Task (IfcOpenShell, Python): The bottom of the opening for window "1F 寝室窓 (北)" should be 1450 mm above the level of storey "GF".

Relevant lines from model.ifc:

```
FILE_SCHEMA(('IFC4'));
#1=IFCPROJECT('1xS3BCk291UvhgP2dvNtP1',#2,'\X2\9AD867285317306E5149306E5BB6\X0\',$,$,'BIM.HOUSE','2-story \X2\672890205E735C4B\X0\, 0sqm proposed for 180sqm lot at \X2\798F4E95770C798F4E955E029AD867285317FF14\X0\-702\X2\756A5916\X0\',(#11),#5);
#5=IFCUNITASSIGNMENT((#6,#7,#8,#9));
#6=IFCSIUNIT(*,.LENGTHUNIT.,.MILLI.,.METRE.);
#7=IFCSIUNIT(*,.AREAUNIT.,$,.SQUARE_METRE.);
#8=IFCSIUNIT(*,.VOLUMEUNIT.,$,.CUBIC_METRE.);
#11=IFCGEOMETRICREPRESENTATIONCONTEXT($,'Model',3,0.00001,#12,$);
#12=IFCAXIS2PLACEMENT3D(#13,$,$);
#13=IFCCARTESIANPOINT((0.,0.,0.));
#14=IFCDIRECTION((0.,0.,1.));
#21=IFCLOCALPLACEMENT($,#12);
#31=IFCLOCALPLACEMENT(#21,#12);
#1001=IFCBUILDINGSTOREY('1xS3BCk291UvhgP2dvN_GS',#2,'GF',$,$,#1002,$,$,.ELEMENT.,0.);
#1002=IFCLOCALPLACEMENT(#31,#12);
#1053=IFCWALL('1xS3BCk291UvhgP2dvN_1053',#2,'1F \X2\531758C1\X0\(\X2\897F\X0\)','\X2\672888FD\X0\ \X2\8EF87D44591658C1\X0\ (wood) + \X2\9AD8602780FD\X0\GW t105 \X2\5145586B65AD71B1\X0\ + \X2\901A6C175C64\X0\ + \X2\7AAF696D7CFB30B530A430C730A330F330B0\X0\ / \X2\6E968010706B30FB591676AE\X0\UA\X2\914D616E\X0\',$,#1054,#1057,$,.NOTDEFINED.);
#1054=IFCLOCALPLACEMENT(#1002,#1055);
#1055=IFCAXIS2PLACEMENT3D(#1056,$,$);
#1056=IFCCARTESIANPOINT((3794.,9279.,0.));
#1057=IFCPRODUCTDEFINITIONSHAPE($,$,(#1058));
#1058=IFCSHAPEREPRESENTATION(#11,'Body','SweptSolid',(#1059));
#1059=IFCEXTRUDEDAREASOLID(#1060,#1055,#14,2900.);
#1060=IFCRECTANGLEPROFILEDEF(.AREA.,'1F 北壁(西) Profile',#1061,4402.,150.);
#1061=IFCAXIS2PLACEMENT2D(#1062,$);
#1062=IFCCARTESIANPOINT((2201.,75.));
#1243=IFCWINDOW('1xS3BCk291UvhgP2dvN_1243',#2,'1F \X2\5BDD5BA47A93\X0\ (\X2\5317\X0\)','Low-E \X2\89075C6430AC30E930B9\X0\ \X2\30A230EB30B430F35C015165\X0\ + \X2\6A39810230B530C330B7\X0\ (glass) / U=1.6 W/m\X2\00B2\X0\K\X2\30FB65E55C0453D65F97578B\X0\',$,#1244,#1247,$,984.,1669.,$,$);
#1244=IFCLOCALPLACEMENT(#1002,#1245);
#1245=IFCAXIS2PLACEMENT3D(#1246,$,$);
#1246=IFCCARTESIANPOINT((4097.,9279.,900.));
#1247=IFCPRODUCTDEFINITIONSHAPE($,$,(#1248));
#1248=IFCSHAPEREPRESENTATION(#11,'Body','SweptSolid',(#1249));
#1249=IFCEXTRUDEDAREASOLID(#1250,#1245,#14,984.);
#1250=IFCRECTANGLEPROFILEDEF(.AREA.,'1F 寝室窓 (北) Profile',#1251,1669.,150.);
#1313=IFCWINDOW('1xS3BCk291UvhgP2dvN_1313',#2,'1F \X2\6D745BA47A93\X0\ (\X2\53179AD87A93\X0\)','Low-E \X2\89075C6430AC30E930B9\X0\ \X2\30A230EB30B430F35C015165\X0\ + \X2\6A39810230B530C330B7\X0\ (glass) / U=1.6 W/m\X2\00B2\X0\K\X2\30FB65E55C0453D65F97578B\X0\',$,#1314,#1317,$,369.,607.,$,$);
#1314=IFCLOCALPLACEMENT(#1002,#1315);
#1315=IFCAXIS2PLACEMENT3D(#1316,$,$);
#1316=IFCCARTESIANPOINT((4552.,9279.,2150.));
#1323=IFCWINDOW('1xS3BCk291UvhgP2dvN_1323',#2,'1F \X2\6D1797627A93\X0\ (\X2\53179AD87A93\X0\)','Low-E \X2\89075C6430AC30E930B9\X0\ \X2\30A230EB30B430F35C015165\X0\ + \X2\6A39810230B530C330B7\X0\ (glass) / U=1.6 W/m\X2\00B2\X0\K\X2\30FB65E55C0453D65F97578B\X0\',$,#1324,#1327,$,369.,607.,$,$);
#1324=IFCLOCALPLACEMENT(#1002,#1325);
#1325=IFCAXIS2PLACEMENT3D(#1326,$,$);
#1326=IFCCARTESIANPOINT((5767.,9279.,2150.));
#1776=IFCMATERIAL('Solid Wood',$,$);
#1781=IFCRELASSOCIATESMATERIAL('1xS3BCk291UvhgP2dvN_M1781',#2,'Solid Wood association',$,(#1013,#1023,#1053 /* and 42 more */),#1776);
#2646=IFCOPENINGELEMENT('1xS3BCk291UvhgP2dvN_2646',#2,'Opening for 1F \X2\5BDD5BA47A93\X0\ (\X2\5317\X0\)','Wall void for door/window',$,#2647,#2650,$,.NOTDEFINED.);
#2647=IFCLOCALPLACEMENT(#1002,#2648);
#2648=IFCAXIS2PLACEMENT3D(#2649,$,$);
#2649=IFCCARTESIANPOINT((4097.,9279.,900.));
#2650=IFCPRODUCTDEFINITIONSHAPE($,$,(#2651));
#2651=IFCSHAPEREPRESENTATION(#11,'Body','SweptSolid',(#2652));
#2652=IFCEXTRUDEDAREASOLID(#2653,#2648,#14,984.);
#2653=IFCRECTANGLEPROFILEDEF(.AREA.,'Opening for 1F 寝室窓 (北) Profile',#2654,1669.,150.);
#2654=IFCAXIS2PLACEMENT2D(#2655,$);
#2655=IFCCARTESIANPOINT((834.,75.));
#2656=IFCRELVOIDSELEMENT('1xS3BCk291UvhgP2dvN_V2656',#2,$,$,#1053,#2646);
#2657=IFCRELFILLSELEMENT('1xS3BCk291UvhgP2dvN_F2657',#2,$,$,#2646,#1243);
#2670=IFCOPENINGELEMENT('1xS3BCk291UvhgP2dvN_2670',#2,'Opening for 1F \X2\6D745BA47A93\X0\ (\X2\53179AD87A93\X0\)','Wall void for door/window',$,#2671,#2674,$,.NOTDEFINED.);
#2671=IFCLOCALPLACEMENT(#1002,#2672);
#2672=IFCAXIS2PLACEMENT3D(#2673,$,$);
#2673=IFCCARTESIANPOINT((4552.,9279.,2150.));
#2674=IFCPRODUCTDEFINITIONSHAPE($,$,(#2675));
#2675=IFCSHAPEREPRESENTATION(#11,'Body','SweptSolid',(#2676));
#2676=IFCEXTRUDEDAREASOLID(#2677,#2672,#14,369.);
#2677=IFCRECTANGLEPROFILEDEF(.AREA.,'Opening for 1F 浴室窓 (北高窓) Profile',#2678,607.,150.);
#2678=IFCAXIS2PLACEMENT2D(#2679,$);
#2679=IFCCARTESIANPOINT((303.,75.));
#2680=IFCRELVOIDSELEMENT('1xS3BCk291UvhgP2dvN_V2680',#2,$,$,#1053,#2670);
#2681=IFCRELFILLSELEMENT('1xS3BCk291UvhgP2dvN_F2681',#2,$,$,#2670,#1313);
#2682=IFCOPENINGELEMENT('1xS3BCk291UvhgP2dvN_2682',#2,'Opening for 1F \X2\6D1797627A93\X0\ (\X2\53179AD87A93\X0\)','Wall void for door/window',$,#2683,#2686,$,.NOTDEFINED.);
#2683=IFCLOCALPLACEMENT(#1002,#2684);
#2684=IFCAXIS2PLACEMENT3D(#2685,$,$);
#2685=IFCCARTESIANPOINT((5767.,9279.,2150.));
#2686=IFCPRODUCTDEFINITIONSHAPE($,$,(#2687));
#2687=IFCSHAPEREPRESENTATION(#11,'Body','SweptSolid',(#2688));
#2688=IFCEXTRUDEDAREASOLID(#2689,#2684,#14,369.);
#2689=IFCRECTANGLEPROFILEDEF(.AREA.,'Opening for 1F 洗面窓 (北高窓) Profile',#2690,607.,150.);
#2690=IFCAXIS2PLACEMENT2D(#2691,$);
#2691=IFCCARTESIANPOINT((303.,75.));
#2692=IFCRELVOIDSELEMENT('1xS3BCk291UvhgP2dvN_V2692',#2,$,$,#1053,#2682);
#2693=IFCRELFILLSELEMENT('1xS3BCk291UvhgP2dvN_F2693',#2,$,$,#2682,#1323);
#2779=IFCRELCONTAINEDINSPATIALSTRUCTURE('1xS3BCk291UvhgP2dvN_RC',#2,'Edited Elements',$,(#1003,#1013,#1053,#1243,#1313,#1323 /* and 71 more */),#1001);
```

```python
import numpy as np
import ifcopenshell
import ifcopenshell.api.geometry
import ifcopenshell.geom
import ifcopenshell.util.element
import ifcopenshell.util.placement
import ifcopenshell.util.shape
import ifcopenshell.util.unit

model = ifcopenshell.open("model.ifc")
unit_scale = ifcopenshell.util.unit.calculate_unit_scale(model)

window = model.by_id(1243)
opening = window.FillsVoids[0].RelatingOpeningElement
storey = ifcopenshell.util.element.get_container(window, ifc_class="IfcBuildingStorey")
level = ifcopenshell.util.placement.get_local_placement(storey.ObjectPlacement)[2, 3]

# The opening's origin need not be at the sill, so measure its lowest point.
shape = ifcopenshell.geom.create_shape(ifcopenshell.geom.settings(), opening)
bottom = ifcopenshell.util.shape.get_shape_bottom_elevation(shape, shape.geometry) / unit_scale
dz = level + 1.45 / unit_scale - bottom

shift = np.array([0.0, 0.0, dz])
# The window is not placed relative to its opening, so move both.
for product in (opening, window):
    matrix = ifcopenshell.util.placement.get_local_placement(product.ObjectPlacement)
    matrix[:3, 3] += shift
    ifcopenshell.api.geometry.edit_object_placement(model, product=product, matrix=matrix, is_si=False)

print(f"moved by {dz * unit_scale:+.3f} m")

model.write("model-out.ifc")
```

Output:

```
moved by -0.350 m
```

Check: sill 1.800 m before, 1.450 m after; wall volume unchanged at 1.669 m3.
